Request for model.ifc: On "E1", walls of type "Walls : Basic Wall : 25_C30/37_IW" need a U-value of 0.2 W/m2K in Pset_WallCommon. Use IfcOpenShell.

First a look at what the model holds.

```python
import ifcopenshell
import ifcopenshell.util.element

model = ifcopenshell.open("model.ifc")
print(model.schema)
storey = next(s for s in model.by_type("IfcBuildingStorey") if s.Name == "E1")
walls = [e for e in ifcopenshell.util.element.get_decomposition(storey) if e.is_a("IfcWall")]
seen = {}
for e in walls:
    element_type = ifcopenshell.util.element.get_type(e)
    key = (element_type.Name if element_type != e and element_type else None, ifcopenshell.util.element.get_pset(e, "Pset_WallCommon", "ThermalTransmittance"))
    seen[key] = seen.get(key, 0) + 1
for (name, value), count in sorted(seen.items(), key=str):
    print(count, "x", name, "|", value)
```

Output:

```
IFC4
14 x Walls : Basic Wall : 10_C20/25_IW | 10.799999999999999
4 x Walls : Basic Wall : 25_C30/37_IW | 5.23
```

```python
import ifcopenshell
import ifcopenshell.api.pset
import ifcopenshell.util.element

model = ifcopenshell.open("model.ifc")

storey = next(s for s in model.by_type("IfcBuildingStorey") if s.Name == "E1")
walls = [e for e in ifcopenshell.util.element.get_decomposition(storey) if e.is_a("IfcWall")]

count = 0
for e in walls:
    element_type = ifcopenshell.util.element.get_type(e)
    if element_type in (None, e) or element_type.Name != "Walls : Basic Wall : 25_C30/37_IW":
        continue
    # add_pset returns the element's existing set when there is one.
    pset = ifcopenshell.api.pset.add_pset(model, product=e, name="Pset_WallCommon")
    ifcopenshell.api.pset.edit_pset(model, pset=pset, properties={"ThermalTransmittance": 0.2})
    count += 1

print(count, "walls updated")

model.write("model-out.ifc")
```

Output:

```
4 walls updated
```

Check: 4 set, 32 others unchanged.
